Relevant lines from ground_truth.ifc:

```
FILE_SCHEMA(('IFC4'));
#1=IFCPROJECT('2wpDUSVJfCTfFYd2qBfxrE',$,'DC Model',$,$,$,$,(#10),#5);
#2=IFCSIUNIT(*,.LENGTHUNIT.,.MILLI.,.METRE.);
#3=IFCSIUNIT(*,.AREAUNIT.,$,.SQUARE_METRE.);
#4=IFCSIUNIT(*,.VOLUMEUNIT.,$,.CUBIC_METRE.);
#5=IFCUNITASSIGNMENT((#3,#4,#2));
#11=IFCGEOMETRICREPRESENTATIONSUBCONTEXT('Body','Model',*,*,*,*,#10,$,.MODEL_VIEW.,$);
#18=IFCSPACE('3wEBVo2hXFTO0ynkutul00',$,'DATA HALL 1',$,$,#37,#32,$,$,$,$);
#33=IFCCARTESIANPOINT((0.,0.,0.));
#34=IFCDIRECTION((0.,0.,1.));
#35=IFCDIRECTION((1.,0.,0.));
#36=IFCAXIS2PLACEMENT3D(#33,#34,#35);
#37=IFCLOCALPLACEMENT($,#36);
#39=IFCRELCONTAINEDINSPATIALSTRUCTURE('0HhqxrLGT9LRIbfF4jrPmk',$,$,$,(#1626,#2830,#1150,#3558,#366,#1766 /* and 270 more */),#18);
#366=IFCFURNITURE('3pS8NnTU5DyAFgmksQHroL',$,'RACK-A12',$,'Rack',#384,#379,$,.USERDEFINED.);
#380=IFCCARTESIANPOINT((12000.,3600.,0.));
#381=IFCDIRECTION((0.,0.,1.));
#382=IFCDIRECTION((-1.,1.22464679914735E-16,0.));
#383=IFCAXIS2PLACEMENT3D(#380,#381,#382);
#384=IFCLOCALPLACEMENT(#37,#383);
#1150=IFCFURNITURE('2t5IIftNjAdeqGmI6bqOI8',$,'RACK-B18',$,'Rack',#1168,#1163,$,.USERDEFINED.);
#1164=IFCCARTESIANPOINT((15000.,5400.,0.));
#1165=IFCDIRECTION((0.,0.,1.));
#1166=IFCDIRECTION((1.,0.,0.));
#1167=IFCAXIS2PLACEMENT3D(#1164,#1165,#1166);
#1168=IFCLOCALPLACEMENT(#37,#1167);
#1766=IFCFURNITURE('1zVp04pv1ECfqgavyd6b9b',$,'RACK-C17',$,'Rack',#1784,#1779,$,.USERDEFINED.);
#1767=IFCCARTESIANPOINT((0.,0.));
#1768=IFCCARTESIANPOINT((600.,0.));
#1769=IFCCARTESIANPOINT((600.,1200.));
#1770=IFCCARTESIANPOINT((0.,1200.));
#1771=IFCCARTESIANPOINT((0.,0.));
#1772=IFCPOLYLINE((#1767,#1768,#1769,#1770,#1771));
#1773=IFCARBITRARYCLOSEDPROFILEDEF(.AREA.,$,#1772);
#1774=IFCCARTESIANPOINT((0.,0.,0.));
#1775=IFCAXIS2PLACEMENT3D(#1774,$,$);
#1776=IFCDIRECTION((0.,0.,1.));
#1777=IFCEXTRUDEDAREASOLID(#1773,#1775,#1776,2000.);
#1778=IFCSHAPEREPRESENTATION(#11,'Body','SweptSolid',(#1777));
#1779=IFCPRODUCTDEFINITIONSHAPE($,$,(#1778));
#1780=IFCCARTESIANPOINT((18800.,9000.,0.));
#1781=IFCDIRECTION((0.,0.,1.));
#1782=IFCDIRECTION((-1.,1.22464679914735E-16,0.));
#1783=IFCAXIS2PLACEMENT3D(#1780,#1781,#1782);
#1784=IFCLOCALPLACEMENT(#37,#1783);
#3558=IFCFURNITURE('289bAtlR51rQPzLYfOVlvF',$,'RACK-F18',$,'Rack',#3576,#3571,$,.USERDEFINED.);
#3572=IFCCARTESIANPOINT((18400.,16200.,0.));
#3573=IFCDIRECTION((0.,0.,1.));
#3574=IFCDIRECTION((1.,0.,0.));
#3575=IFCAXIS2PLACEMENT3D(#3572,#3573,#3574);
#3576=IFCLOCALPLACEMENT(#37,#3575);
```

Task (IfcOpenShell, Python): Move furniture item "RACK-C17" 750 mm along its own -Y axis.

```python
import ifcopenshell
import ifcopenshell.api.geometry
import ifcopenshell.util.placement
import ifcopenshell.util.unit

model = ifcopenshell.open("ground_truth.ifc")
unit_scale = ifcopenshell.util.unit.calculate_unit_scale(model)

item = model.by_guid("1zVp04pv1ECfqgavyd6b9b")
matrix = ifcopenshell.util.placement.get_local_placement(item.ObjectPlacement)
matrix[:3, 3] -= matrix[:3, 1] * 0.75 / unit_scale
ifcopenshell.api.geometry.edit_object_placement(model, product=item, matrix=matrix, is_si=False)

print(ifcopenshell.util.placement.get_local_placement(item.ObjectPlacement).round(3) + 0.0)

model.write("ground_truth_updated.ifc")
```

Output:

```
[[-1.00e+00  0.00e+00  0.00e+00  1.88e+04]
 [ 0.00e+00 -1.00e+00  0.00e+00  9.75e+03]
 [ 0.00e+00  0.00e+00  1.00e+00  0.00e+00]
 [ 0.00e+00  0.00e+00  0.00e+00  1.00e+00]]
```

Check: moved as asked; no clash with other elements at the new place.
